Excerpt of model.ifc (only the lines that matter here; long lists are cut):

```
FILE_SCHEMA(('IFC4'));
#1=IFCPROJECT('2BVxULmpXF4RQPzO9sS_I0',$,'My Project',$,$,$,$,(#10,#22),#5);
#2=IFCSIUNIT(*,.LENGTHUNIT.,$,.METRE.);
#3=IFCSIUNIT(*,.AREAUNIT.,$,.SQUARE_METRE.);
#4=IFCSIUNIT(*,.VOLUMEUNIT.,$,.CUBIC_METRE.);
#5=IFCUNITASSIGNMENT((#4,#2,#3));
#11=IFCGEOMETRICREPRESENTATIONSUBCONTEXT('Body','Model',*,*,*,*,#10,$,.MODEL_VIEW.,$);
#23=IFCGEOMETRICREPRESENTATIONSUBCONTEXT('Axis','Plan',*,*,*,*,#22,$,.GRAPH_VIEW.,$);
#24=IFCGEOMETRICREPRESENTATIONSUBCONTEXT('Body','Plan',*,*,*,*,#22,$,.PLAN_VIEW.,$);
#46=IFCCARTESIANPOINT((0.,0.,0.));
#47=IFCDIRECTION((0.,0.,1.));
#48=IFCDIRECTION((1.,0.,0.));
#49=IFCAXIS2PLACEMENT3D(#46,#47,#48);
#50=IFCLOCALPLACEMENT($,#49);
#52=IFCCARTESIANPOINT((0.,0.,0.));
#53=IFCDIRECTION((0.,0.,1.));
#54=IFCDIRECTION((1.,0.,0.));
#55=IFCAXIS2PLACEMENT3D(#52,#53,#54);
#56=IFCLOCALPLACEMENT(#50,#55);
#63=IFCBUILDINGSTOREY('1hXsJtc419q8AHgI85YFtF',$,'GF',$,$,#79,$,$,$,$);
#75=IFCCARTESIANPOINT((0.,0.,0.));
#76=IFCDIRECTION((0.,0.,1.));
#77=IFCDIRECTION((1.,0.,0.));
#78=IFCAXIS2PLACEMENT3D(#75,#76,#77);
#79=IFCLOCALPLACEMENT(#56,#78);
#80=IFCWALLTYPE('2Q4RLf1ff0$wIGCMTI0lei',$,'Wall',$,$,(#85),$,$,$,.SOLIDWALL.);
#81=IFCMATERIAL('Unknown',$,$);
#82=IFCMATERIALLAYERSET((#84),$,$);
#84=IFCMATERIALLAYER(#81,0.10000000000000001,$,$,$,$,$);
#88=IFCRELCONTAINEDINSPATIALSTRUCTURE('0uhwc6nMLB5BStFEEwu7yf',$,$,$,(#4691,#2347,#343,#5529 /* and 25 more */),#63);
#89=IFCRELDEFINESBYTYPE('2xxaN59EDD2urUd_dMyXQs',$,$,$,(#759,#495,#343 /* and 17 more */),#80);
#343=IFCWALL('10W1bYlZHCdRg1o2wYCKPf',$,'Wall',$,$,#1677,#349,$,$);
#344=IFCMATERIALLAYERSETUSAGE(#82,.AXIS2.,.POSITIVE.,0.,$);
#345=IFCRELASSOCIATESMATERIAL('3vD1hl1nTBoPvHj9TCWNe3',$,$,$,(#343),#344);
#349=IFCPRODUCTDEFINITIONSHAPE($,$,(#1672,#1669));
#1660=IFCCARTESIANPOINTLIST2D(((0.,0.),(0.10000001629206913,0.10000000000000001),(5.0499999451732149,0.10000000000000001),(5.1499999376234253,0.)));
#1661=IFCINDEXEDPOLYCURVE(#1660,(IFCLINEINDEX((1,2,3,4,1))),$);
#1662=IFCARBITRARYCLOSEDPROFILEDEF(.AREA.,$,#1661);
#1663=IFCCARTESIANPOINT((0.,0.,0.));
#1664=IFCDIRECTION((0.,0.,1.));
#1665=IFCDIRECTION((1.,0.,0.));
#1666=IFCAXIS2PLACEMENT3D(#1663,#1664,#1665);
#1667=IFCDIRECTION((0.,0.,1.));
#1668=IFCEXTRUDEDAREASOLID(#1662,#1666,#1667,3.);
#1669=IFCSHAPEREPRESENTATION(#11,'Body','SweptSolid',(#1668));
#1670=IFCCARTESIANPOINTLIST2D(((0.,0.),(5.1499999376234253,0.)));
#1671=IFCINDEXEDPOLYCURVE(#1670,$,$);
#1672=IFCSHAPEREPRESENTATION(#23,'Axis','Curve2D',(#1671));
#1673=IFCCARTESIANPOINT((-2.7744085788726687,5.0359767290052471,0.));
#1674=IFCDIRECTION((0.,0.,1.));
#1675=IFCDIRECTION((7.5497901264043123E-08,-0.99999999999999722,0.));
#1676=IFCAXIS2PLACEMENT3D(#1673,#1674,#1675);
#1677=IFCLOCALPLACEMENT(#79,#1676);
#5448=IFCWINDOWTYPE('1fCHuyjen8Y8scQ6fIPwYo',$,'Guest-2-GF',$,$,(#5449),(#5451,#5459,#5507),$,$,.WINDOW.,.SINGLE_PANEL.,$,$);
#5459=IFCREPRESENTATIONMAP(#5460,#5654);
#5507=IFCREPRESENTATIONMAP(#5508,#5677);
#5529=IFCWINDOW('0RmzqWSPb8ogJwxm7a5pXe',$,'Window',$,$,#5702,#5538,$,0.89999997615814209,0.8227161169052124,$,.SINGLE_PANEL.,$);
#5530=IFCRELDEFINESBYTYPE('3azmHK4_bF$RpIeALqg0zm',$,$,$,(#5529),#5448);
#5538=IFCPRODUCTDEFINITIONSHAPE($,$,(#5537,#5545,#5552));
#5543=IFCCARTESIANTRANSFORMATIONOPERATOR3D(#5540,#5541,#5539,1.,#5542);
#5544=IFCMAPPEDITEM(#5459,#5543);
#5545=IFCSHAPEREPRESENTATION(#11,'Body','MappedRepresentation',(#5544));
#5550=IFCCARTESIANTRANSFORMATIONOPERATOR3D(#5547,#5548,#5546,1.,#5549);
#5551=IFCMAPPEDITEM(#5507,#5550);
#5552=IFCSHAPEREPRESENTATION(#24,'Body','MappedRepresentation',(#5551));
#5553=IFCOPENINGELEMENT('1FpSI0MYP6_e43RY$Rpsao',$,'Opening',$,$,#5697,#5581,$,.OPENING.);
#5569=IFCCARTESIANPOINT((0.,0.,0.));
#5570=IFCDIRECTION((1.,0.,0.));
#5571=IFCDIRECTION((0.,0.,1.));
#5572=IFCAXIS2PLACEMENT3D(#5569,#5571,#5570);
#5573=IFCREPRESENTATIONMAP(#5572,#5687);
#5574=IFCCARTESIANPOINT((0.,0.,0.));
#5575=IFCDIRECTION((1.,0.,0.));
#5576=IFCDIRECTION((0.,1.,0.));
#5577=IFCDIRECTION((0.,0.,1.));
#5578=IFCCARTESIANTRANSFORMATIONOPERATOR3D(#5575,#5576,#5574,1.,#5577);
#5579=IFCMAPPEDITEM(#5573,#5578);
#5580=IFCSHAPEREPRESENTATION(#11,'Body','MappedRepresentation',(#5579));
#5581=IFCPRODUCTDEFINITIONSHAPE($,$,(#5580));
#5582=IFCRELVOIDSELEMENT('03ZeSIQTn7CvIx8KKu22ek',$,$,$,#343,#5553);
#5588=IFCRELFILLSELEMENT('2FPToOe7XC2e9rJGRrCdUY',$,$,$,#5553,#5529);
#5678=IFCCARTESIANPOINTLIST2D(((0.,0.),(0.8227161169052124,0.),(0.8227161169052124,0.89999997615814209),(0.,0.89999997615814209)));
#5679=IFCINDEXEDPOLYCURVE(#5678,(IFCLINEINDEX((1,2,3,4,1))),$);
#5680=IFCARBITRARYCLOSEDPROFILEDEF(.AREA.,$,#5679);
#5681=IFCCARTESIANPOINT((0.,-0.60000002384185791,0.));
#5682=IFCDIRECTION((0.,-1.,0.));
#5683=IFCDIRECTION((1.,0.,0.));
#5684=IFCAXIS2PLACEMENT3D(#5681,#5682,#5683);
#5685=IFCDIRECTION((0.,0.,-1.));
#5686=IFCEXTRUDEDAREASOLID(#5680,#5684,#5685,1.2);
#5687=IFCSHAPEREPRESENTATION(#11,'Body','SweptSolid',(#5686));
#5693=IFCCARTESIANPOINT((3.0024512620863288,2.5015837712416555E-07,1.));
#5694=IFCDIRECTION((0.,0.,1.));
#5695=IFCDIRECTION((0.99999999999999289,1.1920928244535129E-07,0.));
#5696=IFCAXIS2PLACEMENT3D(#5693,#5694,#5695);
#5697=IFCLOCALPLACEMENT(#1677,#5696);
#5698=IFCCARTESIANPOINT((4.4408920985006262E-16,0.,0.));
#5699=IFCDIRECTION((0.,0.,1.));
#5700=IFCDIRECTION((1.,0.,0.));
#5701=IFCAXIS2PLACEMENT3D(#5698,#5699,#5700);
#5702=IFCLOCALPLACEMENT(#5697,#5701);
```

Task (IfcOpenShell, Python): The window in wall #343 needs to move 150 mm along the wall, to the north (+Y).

```python
import ifcopenshell
import ifcopenshell.api.geometry
import ifcopenshell.util.placement
import ifcopenshell.util.unit

model = ifcopenshell.open("model.ifc")
unit_scale = ifcopenshell.util.unit.calculate_unit_scale(model)

window = model.by_guid("0RmzqWSPb8ogJwxm7a5pXe")
opening = window.FillsVoids[0].RelatingOpeningElement
wall = opening.VoidsElements[0].RelatingBuildingElement

wall_matrix = ifcopenshell.util.placement.get_local_placement(wall.ObjectPlacement)
shift = wall_matrix[:3, 0] * -0.15 / unit_scale
before = ifcopenshell.util.placement.get_local_placement(window.ObjectPlacement)[:3, 3].copy()

# The window is placed relative to its opening, so it follows when the opening moves.
matrix = ifcopenshell.util.placement.get_local_placement(opening.ObjectPlacement)
matrix[:3, 3] += shift
ifcopenshell.api.geometry.edit_object_placement(
    model, product=opening, matrix=matrix, is_si=False, should_transform_children=True
)

after = ifcopenshell.util.placement.get_local_placement(window.ObjectPlacement)[:3, 3]
print("window moved by", (after - before).round(3) + 0.0)

model.write("model_rev.ifc")
```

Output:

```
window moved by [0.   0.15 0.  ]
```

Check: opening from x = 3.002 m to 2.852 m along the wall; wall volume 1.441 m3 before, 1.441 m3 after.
